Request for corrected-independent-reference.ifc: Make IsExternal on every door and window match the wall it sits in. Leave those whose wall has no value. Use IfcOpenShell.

First a look at what the model holds.

```python
import ifcopenshell
import ifcopenshell.util.element

model = ifcopenshell.open("corrected-independent-reference.ifc")
print(model.schema)
seen = {}
for e in model.by_type("IfcDoor") + model.by_type("IfcWindow"):
    if not e.FillsVoids:
        continue
    host = e.FillsVoids[0].RelatingOpeningElement.VoidsElements[0].RelatingBuildingElement
    own = ifcopenshell.util.element.get_pset(e, f"Pset_{e.is_a()[3:].removesuffix('StandardCase')}Common", "IsExternal")
    wall = ifcopenshell.util.element.get_pset(host, "Pset_WallCommon", "IsExternal")
    seen[e.is_a(), own, wall] = seen.get((e.is_a(), own, wall), 0) + 1
for (cls, own, wall), count in sorted(seen.items(), key=str):
    print(count, cls, "IsExternal:", own, "| host wall:", wall)
```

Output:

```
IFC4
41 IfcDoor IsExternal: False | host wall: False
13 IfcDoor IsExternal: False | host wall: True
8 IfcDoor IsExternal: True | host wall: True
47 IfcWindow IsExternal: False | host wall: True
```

```python
import ifcopenshell
import ifcopenshell.api.pset
import ifcopenshell.util.element

model = ifcopenshell.open("corrected-independent-reference.ifc")

count = 0
for ifc_class, pset_name in (("IfcDoor", "Pset_DoorCommon"), ("IfcWindow", "Pset_WindowCommon")):
    for e in model.by_type(ifc_class):
        if not e.FillsVoids:
            continue
        host = e.FillsVoids[0].RelatingOpeningElement.VoidsElements[0].RelatingBuildingElement
        external = ifcopenshell.util.element.get_pset(host, "Pset_WallCommon", "IsExternal")
        if external is None or ifcopenshell.util.element.get_pset(e, pset_name, "IsExternal") == external:
            continue
        pset = ifcopenshell.api.pset.add_pset(model, product=e, name=pset_name)
        ifcopenshell.api.pset.edit_pset(model, pset=pset, properties={"IsExternal": external})
        count += 1

print(count, "updated")

model.write("corrected-independent-reference-out.ifc")
```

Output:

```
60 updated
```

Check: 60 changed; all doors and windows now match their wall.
